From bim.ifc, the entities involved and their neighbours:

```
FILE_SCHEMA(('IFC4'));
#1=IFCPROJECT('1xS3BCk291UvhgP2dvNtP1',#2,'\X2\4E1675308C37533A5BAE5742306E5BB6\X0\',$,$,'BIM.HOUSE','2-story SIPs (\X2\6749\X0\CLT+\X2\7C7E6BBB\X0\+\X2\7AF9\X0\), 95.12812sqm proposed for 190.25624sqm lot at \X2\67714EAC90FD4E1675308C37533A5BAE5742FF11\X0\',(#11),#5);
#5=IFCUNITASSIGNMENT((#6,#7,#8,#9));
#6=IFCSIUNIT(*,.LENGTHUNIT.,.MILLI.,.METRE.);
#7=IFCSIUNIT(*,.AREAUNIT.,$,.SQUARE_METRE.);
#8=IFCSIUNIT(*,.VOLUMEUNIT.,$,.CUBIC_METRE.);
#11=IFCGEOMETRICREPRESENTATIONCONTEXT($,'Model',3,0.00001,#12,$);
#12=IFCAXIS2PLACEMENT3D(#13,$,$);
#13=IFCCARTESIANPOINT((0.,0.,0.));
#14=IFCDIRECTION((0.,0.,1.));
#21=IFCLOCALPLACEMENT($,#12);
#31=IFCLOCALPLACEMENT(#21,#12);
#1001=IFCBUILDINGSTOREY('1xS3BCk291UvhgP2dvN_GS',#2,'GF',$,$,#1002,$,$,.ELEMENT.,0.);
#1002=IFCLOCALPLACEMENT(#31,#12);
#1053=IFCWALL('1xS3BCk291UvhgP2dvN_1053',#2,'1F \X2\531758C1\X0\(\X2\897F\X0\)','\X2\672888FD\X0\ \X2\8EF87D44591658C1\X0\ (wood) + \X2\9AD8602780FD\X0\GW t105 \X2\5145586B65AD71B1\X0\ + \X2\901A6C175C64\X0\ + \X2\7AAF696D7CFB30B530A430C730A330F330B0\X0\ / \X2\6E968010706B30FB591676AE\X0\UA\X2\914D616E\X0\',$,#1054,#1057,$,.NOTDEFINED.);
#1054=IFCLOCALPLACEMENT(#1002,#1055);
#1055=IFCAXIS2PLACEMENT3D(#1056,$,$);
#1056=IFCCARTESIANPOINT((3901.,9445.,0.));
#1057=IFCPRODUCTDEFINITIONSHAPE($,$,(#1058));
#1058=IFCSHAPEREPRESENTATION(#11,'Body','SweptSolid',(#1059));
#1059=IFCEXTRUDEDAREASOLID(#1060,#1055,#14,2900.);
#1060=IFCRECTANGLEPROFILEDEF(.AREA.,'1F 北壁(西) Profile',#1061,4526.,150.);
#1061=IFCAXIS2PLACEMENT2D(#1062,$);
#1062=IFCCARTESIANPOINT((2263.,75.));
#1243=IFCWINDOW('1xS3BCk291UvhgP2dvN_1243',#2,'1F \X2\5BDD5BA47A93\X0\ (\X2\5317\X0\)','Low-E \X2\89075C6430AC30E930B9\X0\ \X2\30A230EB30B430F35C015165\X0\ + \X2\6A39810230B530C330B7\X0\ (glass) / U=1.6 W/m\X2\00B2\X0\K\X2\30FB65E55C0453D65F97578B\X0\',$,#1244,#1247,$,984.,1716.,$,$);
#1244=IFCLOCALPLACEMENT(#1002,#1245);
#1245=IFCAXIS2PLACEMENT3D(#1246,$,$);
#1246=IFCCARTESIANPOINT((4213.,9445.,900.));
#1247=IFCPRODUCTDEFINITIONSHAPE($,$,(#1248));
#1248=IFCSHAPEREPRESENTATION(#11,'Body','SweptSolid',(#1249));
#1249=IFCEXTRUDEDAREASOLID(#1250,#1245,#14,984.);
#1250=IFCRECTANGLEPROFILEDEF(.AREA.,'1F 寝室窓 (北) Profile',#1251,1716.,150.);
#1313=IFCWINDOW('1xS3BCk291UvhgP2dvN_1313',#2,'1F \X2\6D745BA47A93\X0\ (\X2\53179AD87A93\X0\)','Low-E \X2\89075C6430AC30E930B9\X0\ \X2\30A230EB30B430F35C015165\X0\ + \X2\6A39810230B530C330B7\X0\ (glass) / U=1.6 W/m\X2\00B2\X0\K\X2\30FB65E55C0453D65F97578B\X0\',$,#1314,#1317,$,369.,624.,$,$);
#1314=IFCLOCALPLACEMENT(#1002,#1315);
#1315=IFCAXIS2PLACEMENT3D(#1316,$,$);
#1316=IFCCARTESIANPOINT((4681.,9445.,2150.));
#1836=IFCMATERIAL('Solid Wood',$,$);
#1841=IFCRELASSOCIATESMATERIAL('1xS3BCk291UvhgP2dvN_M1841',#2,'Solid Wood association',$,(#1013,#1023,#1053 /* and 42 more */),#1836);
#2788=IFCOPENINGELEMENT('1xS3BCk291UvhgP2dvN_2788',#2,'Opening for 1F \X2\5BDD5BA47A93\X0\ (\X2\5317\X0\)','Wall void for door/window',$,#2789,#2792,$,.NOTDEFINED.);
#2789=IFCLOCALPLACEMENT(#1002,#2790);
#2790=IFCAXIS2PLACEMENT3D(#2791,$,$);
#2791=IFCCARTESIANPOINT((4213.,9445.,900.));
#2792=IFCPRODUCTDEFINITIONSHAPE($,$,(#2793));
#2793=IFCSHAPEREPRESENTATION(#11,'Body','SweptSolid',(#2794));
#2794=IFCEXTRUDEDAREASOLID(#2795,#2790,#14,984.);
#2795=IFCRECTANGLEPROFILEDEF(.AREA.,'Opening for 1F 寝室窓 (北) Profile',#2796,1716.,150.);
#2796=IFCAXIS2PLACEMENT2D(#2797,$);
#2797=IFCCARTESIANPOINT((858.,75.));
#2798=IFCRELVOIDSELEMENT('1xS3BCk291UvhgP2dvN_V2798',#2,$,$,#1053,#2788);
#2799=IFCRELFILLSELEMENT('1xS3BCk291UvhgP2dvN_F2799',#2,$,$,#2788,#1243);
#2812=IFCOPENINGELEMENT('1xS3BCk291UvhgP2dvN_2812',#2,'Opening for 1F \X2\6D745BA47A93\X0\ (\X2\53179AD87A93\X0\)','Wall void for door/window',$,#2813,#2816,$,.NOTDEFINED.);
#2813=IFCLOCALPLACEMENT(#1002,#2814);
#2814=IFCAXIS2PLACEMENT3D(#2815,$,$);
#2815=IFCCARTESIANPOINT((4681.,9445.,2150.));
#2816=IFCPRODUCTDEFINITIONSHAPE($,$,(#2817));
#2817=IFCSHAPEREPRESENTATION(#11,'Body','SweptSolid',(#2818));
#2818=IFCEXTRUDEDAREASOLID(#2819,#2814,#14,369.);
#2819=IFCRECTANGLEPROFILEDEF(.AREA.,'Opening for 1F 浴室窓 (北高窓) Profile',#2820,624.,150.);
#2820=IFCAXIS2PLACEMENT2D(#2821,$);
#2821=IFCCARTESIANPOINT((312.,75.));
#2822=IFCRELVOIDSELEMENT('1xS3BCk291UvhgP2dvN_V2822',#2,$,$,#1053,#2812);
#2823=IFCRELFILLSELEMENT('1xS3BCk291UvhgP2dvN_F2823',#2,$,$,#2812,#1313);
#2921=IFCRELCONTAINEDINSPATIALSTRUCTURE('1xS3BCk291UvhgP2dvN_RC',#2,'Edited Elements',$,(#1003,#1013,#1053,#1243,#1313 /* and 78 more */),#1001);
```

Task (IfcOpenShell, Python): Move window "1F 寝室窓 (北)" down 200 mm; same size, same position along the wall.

```python
import numpy as np
import ifcopenshell
import ifcopenshell.api.geometry
import ifcopenshell.util.placement
import ifcopenshell.util.unit

model = ifcopenshell.open("bim.ifc")
unit_scale = ifcopenshell.util.unit.calculate_unit_scale(model)

window = model.by_guid("1xS3BCk291UvhgP2dvN_1243")
opening = window.FillsVoids[0].RelatingOpeningElement
dz = -0.2 / unit_scale

shift = np.array([0.0, 0.0, dz])
# The window is not placed relative to its opening, so move both.
for product in (opening, window):
    matrix = ifcopenshell.util.placement.get_local_placement(product.ObjectPlacement)
    matrix[:3, 3] += shift
    ifcopenshell.api.geometry.edit_object_placement(model, product=product, matrix=matrix, is_si=False)

print(f"moved by {dz * unit_scale:+.3f} m")

model.write("bim_rev.ifc")
```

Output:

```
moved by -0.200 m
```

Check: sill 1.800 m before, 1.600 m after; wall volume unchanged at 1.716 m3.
